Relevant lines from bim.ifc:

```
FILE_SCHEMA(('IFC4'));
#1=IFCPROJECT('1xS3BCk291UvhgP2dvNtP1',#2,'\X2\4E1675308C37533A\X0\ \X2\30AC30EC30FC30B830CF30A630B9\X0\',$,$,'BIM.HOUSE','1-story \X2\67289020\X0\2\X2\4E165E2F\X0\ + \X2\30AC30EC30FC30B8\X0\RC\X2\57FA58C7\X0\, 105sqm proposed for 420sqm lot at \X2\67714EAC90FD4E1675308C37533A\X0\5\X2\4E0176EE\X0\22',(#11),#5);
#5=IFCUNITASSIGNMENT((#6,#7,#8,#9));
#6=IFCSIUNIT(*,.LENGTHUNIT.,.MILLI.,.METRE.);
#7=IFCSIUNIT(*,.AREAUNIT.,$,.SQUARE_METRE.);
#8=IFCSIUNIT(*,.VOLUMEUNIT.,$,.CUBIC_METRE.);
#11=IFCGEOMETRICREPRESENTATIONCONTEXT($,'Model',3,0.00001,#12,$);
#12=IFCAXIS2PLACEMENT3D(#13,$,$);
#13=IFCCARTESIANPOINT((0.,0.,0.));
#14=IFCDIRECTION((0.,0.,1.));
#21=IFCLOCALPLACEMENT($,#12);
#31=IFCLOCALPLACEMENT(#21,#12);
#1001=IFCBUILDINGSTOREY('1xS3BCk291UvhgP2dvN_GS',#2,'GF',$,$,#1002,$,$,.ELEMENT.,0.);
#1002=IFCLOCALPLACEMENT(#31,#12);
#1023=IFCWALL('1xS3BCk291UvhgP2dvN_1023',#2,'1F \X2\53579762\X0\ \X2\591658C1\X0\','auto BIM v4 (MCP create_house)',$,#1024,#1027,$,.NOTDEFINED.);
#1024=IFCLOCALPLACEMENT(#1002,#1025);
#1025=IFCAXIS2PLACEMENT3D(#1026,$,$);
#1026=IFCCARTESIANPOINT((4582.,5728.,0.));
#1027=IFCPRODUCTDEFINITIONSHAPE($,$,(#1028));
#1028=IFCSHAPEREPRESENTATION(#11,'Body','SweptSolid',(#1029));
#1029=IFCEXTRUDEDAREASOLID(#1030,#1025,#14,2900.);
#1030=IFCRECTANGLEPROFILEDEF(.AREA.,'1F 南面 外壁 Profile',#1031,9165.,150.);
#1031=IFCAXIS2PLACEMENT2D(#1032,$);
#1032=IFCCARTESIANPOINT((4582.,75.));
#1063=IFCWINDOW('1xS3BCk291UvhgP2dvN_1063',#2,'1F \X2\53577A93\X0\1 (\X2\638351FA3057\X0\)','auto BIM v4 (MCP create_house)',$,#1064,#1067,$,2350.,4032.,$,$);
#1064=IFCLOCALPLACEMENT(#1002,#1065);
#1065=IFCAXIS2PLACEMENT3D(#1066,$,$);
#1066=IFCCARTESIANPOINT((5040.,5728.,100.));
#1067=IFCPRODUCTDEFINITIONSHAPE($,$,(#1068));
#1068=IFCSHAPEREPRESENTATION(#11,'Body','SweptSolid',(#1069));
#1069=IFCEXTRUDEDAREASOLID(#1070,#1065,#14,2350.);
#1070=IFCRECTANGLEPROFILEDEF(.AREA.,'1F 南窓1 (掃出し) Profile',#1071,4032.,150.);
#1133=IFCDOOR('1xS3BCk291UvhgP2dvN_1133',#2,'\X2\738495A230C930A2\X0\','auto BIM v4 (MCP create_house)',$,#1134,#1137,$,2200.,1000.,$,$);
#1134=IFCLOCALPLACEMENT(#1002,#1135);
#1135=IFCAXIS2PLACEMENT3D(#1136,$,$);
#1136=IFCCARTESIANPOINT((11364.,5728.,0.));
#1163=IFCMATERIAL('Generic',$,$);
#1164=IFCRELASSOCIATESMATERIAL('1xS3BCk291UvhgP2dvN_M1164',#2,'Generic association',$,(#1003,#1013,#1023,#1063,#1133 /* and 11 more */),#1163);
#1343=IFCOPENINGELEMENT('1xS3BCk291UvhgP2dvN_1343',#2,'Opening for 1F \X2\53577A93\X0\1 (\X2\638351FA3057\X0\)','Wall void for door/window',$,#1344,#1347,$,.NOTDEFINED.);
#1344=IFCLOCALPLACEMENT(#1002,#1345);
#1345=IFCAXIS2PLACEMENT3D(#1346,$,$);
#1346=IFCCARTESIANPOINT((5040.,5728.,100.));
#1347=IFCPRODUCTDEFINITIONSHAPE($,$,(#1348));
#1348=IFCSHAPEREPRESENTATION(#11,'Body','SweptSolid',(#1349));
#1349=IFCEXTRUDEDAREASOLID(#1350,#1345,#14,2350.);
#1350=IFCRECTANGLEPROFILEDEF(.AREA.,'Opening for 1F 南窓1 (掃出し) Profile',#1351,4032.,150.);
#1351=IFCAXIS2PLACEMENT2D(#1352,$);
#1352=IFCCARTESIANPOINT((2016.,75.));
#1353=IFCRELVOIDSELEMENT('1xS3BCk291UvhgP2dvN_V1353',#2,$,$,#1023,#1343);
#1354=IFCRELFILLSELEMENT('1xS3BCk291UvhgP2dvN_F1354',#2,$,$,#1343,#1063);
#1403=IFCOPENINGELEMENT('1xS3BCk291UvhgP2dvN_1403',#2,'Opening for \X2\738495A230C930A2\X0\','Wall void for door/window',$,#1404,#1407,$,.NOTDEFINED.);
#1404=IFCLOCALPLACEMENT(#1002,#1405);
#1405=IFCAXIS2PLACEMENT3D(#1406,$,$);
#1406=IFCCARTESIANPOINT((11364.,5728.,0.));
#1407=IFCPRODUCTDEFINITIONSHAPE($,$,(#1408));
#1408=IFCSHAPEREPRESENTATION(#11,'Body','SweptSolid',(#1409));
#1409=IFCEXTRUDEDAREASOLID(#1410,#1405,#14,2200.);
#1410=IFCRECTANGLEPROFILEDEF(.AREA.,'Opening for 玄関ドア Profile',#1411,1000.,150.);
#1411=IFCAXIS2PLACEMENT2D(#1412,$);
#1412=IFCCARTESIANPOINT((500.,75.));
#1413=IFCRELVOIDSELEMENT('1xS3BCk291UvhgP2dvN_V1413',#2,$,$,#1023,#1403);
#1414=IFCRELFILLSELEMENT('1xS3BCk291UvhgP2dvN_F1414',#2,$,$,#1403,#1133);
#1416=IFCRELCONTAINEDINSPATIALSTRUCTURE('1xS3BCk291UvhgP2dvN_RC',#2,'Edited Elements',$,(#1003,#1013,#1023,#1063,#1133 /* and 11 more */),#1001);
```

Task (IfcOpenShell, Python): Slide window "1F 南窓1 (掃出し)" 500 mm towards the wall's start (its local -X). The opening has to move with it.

```python
import ifcopenshell
import ifcopenshell.api.geometry
import ifcopenshell.util.placement
import ifcopenshell.util.unit

model = ifcopenshell.open("bim.ifc")
unit_scale = ifcopenshell.util.unit.calculate_unit_scale(model)

window = model.by_guid("1xS3BCk291UvhgP2dvN_1063")
opening = window.FillsVoids[0].RelatingOpeningElement
wall = opening.VoidsElements[0].RelatingBuildingElement

wall_matrix = ifcopenshell.util.placement.get_local_placement(wall.ObjectPlacement)
shift = wall_matrix[:3, 0] * -0.5 / unit_scale
before = ifcopenshell.util.placement.get_local_placement(window.ObjectPlacement)[:3, 3].copy()

# The window is not placed relative to its opening, so move both.
for product in (opening, window):
    matrix = ifcopenshell.util.placement.get_local_placement(product.ObjectPlacement)
    matrix[:3, 3] += shift
    ifcopenshell.api.geometry.edit_object_placement(model, product=product, matrix=matrix, is_si=False)

after = ifcopenshell.util.placement.get_local_placement(window.ObjectPlacement)[:3, 3]
print("window moved by", (after - before).round(3) + 0.0)

model.write("bim-out.ifc")
```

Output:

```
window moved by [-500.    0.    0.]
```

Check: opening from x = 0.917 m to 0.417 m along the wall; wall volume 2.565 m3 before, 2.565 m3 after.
